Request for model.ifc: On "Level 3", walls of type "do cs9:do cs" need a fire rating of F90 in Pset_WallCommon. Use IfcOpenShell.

First a look at what the model holds.

```python
import ifcopenshell
import ifcopenshell.util.element

model = ifcopenshell.open("model.ifc")
print(model.schema)
storey = next(s for s in model.by_type("IfcBuildingStorey") if s.Name == "Level 3")
walls = [e for e in ifcopenshell.util.element.get_decomposition(storey) if e.is_a("IfcWall")]
seen = {}
for e in walls:
    element_type = ifcopenshell.util.element.get_type(e)
    key = (element_type.Name if element_type != e and element_type else None, ifcopenshell.util.element.get_pset(e, "Pset_WallCommon", "FireRating"))
    seen[key] = seen.get(key, 0) + 1
for (name, value), count in sorted(seen.items(), key=str):
    print(count, "x", name, "|", value)
```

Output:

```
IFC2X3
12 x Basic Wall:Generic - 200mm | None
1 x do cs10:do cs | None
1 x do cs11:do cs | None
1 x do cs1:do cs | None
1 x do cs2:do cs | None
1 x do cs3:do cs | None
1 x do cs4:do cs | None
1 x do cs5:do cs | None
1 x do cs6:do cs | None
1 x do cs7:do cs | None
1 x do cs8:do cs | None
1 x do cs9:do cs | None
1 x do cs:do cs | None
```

```python
import ifcopenshell
import ifcopenshell.api.pset
import ifcopenshell.util.element

model = ifcopenshell.open("model.ifc")

storey = next(s for s in model.by_type("IfcBuildingStorey") if s.Name == "Level 3")
walls = [e for e in ifcopenshell.util.element.get_decomposition(storey) if e.is_a("IfcWall")]

count = 0
for e in walls:
    element_type = ifcopenshell.util.element.get_type(e)
    if element_type in (None, e) or element_type.Name != "do cs9:do cs":
        continue
    # add_pset returns the element's existing set when there is one.
    pset = ifcopenshell.api.pset.add_pset(model, product=e, name="Pset_WallCommon")
    ifcopenshell.api.pset.edit_pset(model, pset=pset, properties={"FireRating": "F90"})
    count += 1

print(count, "walls updated")

model.write("model_updated.ifc")
```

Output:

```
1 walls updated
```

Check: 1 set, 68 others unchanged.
